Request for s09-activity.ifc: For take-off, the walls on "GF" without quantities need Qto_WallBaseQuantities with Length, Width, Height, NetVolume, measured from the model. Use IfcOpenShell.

First a look at what the model holds.

```python
import ifcopenshell
import ifcopenshell.util.element
import ifcopenshell.util.unit

model = ifcopenshell.open("s09-activity.ifc")
print(model.schema)
for unit_type in ("LENGTHUNIT", "AREAUNIT", "VOLUMEUNIT"):
    print(unit_type, ifcopenshell.util.unit.calculate_unit_scale(model, unit_type))
storey = next(s for s in model.by_type("IfcBuildingStorey") if s.Name == "GF")
walls = [e for e in ifcopenshell.util.element.get_decomposition(storey) if e.is_a("IfcWall")]
for e in sorted(walls, key=lambda e: e.id()):
    print(e.id(), e.is_a(), e.Name, list(ifcopenshell.util.element.get_psets(e, qtos_only=True)), sep=" | ")
```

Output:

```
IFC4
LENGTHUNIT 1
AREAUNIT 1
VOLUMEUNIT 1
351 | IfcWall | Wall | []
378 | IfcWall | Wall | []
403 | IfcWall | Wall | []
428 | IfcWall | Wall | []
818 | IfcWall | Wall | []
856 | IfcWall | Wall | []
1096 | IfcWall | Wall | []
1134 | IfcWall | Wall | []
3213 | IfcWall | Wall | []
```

```python
import ifcopenshell
import ifcopenshell.api.pset
import ifcopenshell.geom
import ifcopenshell.util.element
import ifcopenshell.util.shape
import ifcopenshell.util.unit

model = ifcopenshell.open("s09-activity.ifc")
unit_scale = ifcopenshell.util.unit.calculate_unit_scale(model)
volume_scale = ifcopenshell.util.unit.calculate_unit_scale(model, "VOLUMEUNIT")
settings = ifcopenshell.geom.settings()

storey = next(s for s in model.by_type("IfcBuildingStorey") if s.Name == "GF")
walls = [e for e in ifcopenshell.util.element.get_decomposition(storey) if e.is_a("IfcWall")]

for e in sorted(walls, key=lambda e: e.id()):
    if ifcopenshell.util.element.get_psets(e, qtos_only=True, should_inherit=False):
        continue
    # Geometry comes back in metres, in the element's own axes.
    shape = ifcopenshell.geom.create_shape(settings, e)
    values = {
        "Length": ifcopenshell.util.shape.get_x(shape.geometry) / unit_scale,
        "Width": ifcopenshell.util.shape.get_y(shape.geometry) / unit_scale,
        "Height": ifcopenshell.util.shape.get_z(shape.geometry) / unit_scale,
        "NetVolume": ifcopenshell.util.shape.get_volume(shape.geometry) / volume_scale,
    }
    qto = ifcopenshell.api.pset.add_qto(model, product=e, name="Qto_WallBaseQuantities")
    ifcopenshell.api.pset.edit_qto(model, qto=qto, properties=values)
    print(e.id(), {k: round(v, 3) for k, v in values.items()})

model.write("s09-activity_v2.ifc")
```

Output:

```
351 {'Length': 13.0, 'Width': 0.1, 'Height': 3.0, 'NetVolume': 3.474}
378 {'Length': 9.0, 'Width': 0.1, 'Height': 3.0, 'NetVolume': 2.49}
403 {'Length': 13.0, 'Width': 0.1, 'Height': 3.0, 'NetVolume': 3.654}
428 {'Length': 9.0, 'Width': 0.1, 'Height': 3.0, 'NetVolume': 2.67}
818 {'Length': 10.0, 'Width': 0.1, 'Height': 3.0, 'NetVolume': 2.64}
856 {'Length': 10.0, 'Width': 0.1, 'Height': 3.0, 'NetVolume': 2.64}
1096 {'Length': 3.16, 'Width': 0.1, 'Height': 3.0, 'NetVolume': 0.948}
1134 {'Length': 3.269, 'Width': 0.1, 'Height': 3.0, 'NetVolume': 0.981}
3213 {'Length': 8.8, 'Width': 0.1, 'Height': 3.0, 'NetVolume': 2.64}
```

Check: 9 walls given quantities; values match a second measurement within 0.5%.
